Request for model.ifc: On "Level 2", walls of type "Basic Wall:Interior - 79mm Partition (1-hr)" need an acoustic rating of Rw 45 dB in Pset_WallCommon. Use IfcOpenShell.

First a look at what the model holds.

```python
import ifcopenshell
import ifcopenshell.util.element

model = ifcopenshell.open("model.ifc")
print(model.schema)
storey = next(s for s in model.by_type("IfcBuildingStorey") if s.Name == "Level 2")
walls = [e for e in ifcopenshell.util.element.get_decomposition(storey) if e.is_a("IfcWall")]
seen = {}
for e in walls:
    element_type = ifcopenshell.util.element.get_type(e)
    key = (element_type.Name if element_type != e and element_type else None, ifcopenshell.util.element.get_pset(e, "Pset_WallCommon", "AcousticRating"))
    seen[key] = seen.get(key, 0) + 1
for (name, value), count in sorted(seen.items(), key=str):
    print(count, "x", name, "|", value)
```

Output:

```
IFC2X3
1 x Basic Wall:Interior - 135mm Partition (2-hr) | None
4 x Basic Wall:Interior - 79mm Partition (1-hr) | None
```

```python
import ifcopenshell
import ifcopenshell.api.pset
import ifcopenshell.util.element

model = ifcopenshell.open("model.ifc")

storey = next(s for s in model.by_type("IfcBuildingStorey") if s.Name == "Level 2")
walls = [e for e in ifcopenshell.util.element.get_decomposition(storey) if e.is_a("IfcWall")]

count = 0
for e in walls:
    element_type = ifcopenshell.util.element.get_type(e)
    if element_type in (None, e) or element_type.Name != "Basic Wall:Interior - 79mm Partition (1-hr)":
        continue
    # add_pset returns the element's existing set when there is one.
    pset = ifcopenshell.api.pset.add_pset(model, product=e, name="Pset_WallCommon")
    ifcopenshell.api.pset.edit_pset(model, pset=pset, properties={"AcousticRating": "Rw 45 dB"})
    count += 1

print(count, "walls updated")

model.write("model_updated.ifc")
```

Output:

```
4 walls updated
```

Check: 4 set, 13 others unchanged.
